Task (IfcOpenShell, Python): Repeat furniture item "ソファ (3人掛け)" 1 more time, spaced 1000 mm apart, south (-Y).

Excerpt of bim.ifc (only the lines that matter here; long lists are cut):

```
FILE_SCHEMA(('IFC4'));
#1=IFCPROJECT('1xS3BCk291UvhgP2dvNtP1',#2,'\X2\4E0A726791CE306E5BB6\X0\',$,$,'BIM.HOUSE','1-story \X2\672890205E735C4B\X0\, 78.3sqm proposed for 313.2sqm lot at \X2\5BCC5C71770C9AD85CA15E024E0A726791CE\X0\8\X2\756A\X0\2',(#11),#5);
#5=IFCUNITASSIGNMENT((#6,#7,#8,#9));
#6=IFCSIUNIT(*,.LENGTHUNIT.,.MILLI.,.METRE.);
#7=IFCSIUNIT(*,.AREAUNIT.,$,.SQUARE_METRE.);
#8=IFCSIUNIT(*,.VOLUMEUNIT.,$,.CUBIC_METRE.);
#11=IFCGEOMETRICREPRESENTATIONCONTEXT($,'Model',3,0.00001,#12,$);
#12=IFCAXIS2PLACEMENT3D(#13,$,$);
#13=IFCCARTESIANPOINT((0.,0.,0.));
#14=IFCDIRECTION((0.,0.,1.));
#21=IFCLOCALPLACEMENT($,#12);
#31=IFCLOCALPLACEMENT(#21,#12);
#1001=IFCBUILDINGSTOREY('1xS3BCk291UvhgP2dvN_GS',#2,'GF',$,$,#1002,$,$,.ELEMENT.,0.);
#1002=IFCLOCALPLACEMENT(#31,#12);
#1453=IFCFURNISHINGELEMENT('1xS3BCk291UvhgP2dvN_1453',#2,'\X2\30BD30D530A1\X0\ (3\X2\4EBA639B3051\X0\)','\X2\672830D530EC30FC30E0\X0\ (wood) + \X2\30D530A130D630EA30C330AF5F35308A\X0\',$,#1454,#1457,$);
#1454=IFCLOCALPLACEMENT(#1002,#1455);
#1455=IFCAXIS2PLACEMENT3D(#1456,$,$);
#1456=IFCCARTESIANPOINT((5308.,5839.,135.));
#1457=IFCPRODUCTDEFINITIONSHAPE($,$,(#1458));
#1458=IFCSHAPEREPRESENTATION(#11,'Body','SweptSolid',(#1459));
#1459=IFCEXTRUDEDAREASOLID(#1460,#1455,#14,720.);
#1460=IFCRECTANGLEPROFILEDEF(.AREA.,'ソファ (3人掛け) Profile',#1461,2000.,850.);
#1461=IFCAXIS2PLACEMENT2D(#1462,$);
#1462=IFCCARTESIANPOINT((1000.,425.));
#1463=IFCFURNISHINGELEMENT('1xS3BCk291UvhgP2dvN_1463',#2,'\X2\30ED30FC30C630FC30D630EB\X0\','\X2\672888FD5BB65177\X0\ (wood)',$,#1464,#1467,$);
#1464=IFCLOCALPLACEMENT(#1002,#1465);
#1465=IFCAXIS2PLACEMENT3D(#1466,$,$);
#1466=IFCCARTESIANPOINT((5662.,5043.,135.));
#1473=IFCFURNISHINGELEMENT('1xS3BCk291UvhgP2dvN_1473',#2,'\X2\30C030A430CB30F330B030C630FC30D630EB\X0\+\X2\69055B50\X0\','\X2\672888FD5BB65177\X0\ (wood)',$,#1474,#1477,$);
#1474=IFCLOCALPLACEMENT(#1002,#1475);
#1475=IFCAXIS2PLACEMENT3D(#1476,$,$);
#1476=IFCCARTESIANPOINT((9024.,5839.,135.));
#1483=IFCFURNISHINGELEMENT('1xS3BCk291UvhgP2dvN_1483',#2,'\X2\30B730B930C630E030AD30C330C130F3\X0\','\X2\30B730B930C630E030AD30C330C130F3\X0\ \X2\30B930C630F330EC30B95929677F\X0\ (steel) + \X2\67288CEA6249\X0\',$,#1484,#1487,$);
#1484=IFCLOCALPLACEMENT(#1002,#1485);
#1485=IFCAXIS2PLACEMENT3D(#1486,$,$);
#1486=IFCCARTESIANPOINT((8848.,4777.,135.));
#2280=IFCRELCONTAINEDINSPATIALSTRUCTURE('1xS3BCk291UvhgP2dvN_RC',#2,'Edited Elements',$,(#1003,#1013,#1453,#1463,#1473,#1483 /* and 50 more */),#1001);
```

```python
import numpy as np
import ifcopenshell
import ifcopenshell.api.geometry
import ifcopenshell.api.root
import ifcopenshell.util.element
import ifcopenshell.util.placement
import ifcopenshell.util.unit

model = ifcopenshell.open("bim.ifc")
unit_scale = ifcopenshell.util.unit.calculate_unit_scale(model)


def reuse_history(source, copy):
    """copy_class also copies each property set's owner history, people and application; keep the originals."""
    for rel in copy.IsDefinedBy:
        if rel.is_a("IfcRelDefinesByProperties") and (history := rel.RelatingPropertyDefinition.OwnerHistory):
            rel.RelatingPropertyDefinition.OwnerHistory = source.OwnerHistory
            ifcopenshell.util.element.remove_deep2(model, history)


source = model.by_id(1453)
base = ifcopenshell.util.placement.get_local_placement(source.ObjectPlacement)
step = np.array([0.0, -1.0, 0.0]) * 1 / unit_scale

for i in range(1, 2):
    copy = ifcopenshell.api.root.copy_class(model, product=source)
    copy.Representation = ifcopenshell.util.element.copy_deep(
        model, source.Representation, exclude=["IfcGeometricRepresentationContext", "IfcRepresentationMap"]
    )
    reuse_history(source, copy)
    matrix = base.copy()
    matrix[:3, 3] += i * step
    print("added at", matrix[:3, 3].round(3) + 0.0)
    ifcopenshell.api.geometry.edit_object_placement(model, product=copy, matrix=matrix, is_si=False)

model.write("bim-out.ifc")
```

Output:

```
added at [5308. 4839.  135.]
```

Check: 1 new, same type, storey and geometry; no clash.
